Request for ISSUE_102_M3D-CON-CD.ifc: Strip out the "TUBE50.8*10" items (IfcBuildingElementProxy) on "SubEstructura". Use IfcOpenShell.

First a look at what the model holds.

```python
import ifcopenshell
import ifcopenshell.util.element

model = ifcopenshell.open("ISSUE_102_M3D-CON-CD.ifc")
print(model.schema)
storey = next(s for s in model.by_type("IfcBuildingStorey") if s.Name == "SubEstructura")
proxies = [e for e in ifcopenshell.util.element.get_decomposition(storey) if e.is_a("IfcBuildingElementProxy")]
seen = {}
for e in proxies:
    element_type = ifcopenshell.util.element.get_type(e)
    name = element_type.Name if element_type not in (None, e) else None
    seen[name] = seen.get(name, 0) + 1
for name, count in sorted(seen.items(), key=str):
    print(count, "x", name)
```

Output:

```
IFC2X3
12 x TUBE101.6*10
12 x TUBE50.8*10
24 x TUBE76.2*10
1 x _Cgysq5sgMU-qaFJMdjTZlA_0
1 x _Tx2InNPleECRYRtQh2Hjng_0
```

```python
import ifcopenshell
import ifcopenshell.api.root
import ifcopenshell.util.element

model = ifcopenshell.open("ISSUE_102_M3D-CON-CD.ifc")

storey = next(s for s in model.by_type("IfcBuildingStorey") if s.Name == "SubEstructura")
proxies = [e for e in ifcopenshell.util.element.get_decomposition(storey) if e.is_a("IfcBuildingElementProxy")]
targets = [e for e in proxies if (t := ifcopenshell.util.element.get_type(e)) not in (None, e) and t.Name == "TUBE50.8*10"]

for e in targets:
    ifcopenshell.api.root.remove_product(model, product=e)
print(len(targets), "removed")

model.write("ISSUE_102_M3D-CON-CD_v2.ifc")
```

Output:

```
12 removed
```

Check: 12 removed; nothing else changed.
